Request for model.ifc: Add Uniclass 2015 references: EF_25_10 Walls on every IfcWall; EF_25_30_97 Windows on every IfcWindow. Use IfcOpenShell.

First a look at what the model holds.

```python
import ifcopenshell

model = ifcopenshell.open("model.ifc")
print(model.schema)
print("classifications:", [c.Name for c in model.by_type("IfcClassification")])
for ifc_class in ("IfcDoor", "IfcRoof", "IfcStair", "IfcWall", "IfcWindow"):
    print(ifc_class, len(model.by_type(ifc_class)))
```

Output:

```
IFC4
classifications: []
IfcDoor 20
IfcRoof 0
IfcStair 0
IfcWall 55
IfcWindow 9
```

```python
import ifcopenshell
import ifcopenshell.api.classification

model = ifcopenshell.open("model.ifc")

system = ifcopenshell.api.classification.add_classification(model, classification="Uniclass 2015")

codes = {
    "IfcWall": ("EF_25_10", "Walls"),
    "IfcWindow": ("EF_25_30_97", "Windows"),
}
for ifc_class, (code, name) in codes.items():
    products = model.by_type(ifc_class)
    ifcopenshell.api.classification.add_reference(
        model, products=products, classification=system, identification=code, name=name
    )
    print(code, len(products))

model.write("model-out.ifc")
```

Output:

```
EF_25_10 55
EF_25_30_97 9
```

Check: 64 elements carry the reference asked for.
